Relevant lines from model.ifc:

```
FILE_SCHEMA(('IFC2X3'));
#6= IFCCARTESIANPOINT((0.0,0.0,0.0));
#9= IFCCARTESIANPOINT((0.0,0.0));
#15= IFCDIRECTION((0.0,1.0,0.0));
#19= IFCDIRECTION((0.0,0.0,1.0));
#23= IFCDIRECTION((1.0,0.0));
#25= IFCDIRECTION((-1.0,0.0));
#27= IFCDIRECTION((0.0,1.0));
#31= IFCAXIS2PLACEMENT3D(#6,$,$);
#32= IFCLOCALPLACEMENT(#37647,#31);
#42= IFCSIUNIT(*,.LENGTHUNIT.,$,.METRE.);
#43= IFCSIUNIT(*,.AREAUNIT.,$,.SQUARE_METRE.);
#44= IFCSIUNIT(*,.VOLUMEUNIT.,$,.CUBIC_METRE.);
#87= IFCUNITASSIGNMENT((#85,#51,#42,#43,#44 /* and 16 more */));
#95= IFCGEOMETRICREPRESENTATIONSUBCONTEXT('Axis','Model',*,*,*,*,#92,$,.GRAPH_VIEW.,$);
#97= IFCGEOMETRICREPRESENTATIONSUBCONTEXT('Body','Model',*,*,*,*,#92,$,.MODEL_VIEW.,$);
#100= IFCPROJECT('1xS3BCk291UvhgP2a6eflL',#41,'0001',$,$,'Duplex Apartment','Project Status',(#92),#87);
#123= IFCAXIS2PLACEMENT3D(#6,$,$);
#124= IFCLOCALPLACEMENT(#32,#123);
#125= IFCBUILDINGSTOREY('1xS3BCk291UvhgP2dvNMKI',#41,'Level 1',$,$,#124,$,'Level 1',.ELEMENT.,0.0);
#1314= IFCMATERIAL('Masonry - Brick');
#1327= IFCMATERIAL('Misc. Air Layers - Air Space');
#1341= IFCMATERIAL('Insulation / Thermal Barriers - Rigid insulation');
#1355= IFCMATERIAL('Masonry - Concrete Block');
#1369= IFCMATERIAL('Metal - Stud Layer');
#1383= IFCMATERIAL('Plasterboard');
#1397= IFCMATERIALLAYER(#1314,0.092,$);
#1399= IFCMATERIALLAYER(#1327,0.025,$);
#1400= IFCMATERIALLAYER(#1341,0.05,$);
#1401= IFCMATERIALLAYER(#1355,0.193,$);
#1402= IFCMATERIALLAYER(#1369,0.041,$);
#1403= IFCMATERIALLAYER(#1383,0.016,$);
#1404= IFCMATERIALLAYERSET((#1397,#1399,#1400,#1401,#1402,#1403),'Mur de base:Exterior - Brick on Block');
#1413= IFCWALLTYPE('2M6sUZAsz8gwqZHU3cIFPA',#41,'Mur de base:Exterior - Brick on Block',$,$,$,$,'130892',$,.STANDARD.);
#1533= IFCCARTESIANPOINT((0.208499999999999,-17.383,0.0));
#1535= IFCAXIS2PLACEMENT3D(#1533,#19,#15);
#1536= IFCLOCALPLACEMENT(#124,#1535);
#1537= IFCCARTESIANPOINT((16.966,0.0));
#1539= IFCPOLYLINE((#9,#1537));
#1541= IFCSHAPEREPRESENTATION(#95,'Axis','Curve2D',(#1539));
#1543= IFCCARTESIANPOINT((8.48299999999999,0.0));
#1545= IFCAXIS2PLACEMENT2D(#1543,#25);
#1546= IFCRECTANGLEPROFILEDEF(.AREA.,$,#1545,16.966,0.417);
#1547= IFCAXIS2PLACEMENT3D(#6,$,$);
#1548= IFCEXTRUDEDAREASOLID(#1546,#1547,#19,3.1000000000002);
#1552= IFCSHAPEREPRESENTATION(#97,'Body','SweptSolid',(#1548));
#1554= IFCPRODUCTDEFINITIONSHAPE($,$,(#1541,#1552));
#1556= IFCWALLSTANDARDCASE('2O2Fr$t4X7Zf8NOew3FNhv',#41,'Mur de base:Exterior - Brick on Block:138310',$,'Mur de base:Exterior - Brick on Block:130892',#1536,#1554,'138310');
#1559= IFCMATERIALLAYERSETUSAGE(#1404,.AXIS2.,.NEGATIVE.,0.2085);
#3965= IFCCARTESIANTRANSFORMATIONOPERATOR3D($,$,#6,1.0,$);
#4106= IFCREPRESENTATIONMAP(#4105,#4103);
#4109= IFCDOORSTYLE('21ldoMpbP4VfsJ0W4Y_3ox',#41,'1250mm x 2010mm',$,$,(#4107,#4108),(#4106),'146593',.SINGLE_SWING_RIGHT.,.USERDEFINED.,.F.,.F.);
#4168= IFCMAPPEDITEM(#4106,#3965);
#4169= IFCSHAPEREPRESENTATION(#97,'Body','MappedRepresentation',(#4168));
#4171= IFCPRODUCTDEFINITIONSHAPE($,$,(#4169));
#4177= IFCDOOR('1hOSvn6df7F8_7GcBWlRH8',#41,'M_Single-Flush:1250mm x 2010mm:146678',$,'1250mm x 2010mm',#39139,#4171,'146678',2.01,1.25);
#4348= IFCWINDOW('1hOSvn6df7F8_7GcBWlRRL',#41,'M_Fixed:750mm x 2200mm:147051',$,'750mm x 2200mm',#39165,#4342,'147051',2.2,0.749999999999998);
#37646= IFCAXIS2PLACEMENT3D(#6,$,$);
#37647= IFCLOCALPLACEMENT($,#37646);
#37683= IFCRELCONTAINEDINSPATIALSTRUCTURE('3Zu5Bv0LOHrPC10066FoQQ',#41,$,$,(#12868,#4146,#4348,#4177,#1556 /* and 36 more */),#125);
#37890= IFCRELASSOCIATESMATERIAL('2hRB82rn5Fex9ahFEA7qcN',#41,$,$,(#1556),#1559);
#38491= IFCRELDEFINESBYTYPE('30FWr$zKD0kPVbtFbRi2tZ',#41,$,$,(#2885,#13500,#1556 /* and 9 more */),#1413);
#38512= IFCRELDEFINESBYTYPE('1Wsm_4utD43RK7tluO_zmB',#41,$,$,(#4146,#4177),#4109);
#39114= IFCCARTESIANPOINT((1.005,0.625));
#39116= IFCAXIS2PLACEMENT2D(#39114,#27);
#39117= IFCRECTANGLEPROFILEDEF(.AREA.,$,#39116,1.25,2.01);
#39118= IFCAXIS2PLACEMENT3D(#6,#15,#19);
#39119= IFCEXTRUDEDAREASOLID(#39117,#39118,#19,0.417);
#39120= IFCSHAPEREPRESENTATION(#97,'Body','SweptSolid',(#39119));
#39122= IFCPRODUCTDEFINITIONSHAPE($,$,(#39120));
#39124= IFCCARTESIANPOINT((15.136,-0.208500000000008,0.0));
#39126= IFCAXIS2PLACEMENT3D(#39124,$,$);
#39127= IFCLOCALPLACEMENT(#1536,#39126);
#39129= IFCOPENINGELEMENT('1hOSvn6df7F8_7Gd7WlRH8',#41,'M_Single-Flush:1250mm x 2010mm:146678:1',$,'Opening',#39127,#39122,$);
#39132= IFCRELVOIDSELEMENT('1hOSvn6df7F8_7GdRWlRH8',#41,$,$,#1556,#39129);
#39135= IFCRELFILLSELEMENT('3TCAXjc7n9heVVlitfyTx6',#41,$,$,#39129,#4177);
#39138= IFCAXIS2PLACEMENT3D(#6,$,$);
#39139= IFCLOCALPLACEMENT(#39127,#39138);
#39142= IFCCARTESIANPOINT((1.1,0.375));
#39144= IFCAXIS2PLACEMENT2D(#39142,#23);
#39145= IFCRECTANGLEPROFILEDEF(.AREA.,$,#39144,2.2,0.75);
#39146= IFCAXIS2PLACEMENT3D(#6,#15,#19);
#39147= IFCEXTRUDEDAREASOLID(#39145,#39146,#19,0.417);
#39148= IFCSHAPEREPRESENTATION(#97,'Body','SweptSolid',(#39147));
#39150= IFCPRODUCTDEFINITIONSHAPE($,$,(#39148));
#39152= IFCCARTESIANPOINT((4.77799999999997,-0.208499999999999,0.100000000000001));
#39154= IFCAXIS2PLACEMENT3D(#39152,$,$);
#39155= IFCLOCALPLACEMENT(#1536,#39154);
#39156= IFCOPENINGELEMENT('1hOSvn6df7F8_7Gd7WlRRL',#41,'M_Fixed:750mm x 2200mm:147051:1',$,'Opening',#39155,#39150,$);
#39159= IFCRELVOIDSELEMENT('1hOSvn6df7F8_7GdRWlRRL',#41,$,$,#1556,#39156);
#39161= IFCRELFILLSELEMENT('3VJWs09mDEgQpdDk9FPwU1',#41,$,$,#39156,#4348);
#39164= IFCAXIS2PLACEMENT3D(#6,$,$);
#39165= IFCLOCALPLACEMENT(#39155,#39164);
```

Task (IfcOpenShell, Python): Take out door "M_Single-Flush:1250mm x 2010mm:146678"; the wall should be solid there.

```python
import ifcopenshell
import ifcopenshell.api.feature
import ifcopenshell.api.root
import ifcopenshell.geom
import ifcopenshell.util.shape

model = ifcopenshell.open("model.ifc")
settings = ifcopenshell.geom.settings()


def volume(element):
    """Net volume in cubic metres, openings subtracted."""
    shape = ifcopenshell.geom.create_shape(settings, element)
    return ifcopenshell.util.shape.get_volume(shape.geometry)


door = model.by_id(4177)
opening = door.FillsVoids[0].RelatingOpeningElement
wall = opening.VoidsElements[0].RelatingBuildingElement
before = volume(wall)

ifcopenshell.api.root.remove_product(model, product=door)
ifcopenshell.api.feature.remove_feature(model, feature=opening)

after = volume(wall)

print(f"wall volume {before:.3f} -> {after:.3f} m3")

model.write("model_edited.ifc")
```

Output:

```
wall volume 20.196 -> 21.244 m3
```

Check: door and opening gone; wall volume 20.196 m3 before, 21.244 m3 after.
